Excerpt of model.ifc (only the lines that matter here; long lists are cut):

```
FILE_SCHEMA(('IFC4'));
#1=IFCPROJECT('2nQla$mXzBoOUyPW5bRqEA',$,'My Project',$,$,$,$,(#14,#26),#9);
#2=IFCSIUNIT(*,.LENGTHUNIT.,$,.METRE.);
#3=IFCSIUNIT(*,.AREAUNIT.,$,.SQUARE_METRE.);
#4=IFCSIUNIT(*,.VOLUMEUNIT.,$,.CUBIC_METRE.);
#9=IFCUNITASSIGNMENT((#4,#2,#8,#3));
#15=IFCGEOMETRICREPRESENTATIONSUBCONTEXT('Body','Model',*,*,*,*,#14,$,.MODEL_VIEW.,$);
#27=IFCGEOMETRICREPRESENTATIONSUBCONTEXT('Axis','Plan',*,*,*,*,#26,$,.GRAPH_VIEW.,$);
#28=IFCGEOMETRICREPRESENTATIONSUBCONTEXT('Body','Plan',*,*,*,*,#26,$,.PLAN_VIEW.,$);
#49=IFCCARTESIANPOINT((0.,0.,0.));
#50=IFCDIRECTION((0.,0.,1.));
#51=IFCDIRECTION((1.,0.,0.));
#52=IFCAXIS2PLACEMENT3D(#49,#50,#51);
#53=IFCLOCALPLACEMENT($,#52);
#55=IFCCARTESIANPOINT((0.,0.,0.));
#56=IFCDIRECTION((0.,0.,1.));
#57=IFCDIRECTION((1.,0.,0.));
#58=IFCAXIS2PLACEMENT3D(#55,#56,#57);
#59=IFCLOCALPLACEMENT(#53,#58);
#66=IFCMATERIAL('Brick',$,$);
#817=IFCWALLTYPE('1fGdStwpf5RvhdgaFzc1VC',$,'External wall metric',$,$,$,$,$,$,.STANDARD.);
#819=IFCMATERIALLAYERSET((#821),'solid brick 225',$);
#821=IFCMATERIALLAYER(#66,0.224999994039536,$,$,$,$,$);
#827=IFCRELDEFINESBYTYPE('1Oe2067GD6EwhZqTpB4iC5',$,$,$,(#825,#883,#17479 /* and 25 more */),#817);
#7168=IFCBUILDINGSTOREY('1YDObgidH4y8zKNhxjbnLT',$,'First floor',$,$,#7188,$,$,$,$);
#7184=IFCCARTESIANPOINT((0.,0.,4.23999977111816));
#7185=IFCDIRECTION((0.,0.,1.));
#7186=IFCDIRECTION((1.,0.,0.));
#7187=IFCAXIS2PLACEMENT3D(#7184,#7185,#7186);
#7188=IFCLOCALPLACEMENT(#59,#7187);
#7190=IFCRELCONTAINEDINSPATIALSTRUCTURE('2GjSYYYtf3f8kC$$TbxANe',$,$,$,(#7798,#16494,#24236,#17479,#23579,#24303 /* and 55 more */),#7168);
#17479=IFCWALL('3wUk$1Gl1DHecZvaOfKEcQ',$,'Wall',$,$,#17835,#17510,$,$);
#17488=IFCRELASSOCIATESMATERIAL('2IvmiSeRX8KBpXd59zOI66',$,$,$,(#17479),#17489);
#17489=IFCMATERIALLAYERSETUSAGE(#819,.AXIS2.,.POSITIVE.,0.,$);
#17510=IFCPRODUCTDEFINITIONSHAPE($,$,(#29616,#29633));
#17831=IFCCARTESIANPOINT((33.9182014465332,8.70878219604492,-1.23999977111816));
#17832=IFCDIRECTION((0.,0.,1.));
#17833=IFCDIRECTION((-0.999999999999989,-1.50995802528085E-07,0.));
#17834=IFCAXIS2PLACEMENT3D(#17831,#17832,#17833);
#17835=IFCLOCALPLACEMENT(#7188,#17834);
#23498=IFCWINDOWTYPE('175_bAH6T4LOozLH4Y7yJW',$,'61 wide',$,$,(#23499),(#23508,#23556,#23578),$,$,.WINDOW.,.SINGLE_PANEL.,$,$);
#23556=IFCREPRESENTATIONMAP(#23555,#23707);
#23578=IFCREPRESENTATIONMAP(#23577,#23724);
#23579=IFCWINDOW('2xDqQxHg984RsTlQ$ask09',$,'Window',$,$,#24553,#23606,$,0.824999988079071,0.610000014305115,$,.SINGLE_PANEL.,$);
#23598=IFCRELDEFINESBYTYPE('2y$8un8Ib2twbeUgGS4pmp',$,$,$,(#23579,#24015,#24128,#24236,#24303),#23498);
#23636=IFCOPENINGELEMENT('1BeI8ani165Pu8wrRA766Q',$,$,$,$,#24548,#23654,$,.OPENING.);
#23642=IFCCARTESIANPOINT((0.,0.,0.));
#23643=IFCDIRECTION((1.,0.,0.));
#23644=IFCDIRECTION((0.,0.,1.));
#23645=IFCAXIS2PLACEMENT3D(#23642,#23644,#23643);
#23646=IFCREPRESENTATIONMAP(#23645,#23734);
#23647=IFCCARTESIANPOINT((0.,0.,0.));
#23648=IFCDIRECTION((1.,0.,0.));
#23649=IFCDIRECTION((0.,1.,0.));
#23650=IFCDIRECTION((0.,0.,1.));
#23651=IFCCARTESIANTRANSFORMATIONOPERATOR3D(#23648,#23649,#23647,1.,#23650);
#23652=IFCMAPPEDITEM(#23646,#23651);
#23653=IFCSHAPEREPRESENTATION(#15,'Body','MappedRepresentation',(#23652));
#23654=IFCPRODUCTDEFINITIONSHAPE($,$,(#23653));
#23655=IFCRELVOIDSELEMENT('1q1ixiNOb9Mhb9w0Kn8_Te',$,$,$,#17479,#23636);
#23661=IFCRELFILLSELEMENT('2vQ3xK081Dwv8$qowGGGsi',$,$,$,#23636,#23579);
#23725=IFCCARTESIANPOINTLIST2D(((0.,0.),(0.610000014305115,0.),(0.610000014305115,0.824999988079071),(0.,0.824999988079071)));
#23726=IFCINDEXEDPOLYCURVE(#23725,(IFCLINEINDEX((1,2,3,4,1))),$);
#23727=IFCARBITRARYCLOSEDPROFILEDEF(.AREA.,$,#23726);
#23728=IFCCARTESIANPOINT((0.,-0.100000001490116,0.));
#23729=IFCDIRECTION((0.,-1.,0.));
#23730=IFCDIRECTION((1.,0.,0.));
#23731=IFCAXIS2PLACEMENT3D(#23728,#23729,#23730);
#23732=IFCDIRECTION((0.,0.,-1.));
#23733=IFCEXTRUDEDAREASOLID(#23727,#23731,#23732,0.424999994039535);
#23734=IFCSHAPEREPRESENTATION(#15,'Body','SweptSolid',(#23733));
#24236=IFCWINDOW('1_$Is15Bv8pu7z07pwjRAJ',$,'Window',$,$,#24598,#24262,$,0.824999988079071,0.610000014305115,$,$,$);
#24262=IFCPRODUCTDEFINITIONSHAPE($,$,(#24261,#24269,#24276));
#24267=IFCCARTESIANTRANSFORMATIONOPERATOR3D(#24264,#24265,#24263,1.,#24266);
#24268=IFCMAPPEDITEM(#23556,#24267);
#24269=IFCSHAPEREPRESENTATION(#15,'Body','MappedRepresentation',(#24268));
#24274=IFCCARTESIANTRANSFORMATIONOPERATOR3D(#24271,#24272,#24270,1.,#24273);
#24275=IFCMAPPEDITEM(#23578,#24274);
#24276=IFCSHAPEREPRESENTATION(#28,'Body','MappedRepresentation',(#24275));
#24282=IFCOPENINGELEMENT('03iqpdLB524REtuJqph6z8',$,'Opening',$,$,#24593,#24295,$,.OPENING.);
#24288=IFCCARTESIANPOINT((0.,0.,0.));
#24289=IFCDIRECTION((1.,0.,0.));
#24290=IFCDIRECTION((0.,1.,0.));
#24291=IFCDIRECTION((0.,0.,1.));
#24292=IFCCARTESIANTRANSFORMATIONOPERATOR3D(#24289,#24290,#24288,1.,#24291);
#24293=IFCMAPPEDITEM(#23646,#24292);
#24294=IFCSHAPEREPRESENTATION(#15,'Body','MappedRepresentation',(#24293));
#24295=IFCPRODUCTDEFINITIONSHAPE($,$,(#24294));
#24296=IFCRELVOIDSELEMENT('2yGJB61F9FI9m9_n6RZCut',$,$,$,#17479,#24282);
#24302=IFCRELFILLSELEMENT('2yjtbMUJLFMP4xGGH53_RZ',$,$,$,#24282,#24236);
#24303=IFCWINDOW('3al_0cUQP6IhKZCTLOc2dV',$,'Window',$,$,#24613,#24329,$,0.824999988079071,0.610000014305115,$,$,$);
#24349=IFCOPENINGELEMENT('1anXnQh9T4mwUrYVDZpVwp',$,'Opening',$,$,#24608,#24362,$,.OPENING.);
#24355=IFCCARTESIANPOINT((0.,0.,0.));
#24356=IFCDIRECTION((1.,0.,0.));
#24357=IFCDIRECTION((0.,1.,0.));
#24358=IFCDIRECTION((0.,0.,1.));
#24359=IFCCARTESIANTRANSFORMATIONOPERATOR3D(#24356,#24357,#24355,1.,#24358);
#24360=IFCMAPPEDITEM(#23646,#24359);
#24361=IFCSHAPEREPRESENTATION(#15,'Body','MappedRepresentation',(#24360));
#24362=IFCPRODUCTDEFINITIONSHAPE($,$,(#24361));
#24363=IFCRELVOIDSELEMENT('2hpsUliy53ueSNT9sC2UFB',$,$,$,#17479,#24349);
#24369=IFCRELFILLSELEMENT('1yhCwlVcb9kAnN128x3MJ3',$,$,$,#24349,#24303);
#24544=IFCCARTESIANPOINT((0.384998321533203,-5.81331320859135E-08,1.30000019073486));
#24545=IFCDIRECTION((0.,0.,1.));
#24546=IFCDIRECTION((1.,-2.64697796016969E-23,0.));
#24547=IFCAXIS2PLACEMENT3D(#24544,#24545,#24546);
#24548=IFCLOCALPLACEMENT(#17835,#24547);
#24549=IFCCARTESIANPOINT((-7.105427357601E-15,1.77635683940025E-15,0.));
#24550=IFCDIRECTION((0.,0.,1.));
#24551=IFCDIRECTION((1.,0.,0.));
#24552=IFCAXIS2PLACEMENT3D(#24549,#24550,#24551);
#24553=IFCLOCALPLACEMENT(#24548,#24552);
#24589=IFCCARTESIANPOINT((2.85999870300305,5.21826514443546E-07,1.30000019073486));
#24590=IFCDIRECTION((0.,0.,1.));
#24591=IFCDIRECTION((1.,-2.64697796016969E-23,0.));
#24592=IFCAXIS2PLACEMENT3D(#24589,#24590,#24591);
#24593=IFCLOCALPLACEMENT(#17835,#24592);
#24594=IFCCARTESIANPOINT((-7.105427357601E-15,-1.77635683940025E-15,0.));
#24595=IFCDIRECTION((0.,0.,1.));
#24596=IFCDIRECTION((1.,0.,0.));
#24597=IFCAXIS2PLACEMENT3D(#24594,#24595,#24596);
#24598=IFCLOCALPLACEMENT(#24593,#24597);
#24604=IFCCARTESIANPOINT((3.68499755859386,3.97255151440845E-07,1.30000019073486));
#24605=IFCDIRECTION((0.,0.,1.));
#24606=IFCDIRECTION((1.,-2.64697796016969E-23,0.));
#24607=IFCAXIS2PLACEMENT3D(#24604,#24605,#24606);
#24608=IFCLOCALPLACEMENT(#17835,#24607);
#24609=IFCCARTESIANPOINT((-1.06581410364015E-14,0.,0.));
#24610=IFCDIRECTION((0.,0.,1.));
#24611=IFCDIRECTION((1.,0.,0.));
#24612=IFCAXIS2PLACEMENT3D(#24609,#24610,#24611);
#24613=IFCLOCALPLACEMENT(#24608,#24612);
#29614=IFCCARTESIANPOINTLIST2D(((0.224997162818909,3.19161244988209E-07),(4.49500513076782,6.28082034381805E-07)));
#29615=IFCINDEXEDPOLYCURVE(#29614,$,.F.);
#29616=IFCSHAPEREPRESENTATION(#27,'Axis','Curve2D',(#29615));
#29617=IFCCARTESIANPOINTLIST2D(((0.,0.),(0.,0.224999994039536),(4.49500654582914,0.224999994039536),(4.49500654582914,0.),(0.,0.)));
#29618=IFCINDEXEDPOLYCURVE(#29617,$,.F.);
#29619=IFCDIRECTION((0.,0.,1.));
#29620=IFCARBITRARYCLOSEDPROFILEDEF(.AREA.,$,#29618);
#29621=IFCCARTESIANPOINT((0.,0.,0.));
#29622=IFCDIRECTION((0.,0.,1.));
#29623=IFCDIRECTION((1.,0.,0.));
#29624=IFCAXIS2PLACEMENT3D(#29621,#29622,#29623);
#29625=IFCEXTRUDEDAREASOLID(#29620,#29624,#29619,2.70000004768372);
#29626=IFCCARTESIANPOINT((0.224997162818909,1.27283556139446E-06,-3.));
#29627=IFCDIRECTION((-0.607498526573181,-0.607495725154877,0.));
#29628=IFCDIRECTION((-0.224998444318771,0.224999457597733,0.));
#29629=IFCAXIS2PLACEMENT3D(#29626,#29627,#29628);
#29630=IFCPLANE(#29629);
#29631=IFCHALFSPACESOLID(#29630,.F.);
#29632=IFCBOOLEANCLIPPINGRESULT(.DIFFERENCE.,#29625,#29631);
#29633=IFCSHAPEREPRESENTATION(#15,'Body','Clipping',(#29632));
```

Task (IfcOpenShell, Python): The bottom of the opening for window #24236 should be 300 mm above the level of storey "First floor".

```python
import numpy as np
import ifcopenshell
import ifcopenshell.api.geometry
import ifcopenshell.geom
import ifcopenshell.util.element
import ifcopenshell.util.placement
import ifcopenshell.util.shape
import ifcopenshell.util.unit

model = ifcopenshell.open("model.ifc")
unit_scale = ifcopenshell.util.unit.calculate_unit_scale(model)

window = model.by_guid("1_$Is15Bv8pu7z07pwjRAJ")
opening = window.FillsVoids[0].RelatingOpeningElement
storey = ifcopenshell.util.element.get_container(window, ifc_class="IfcBuildingStorey")
level = ifcopenshell.util.placement.get_local_placement(storey.ObjectPlacement)[2, 3]

# The opening's origin need not be at the sill, so measure its lowest point.
shape = ifcopenshell.geom.create_shape(ifcopenshell.geom.settings(), opening)
bottom = ifcopenshell.util.shape.get_shape_bottom_elevation(shape, shape.geometry) / unit_scale
dz = level + 0.3 - bottom

shift = np.array([0.0, 0.0, dz])
# The window is placed relative to its opening, so it follows when the opening moves.
matrix = ifcopenshell.util.placement.get_local_placement(opening.ObjectPlacement)
matrix[:3, 3] += shift
ifcopenshell.api.geometry.edit_object_placement(
    model, product=opening, matrix=matrix, is_si=False, should_transform_children=True
)

print(f"moved by {dz * unit_scale:+.3f} m")

model.write("model-out.ifc")
```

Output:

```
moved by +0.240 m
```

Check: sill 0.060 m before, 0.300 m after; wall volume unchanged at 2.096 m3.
